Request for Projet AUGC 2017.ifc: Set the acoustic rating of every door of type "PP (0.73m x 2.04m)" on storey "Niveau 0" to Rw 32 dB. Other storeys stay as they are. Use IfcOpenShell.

First a look at what the model holds.

```python
import ifcopenshell
import ifcopenshell.util.element

model = ifcopenshell.open("Projet AUGC 2017.ifc")
print(model.schema)
storey = next(s for s in model.by_type("IfcBuildingStorey") if s.Name == "Niveau 0")
doors = [e for e in ifcopenshell.util.element.get_decomposition(storey) if e.is_a("IfcDoor")]
seen = {}
for e in doors:
    element_type = ifcopenshell.util.element.get_type(e)
    key = (element_type.Name if element_type != e and element_type else None, ifcopenshell.util.element.get_pset(e, "Pset_DoorCommon", "AcousticRating"))
    seen[key] = seen.get(key, 0) + 1
for (name, value), count in sorted(seen.items(), key=str):
    print(count, "x", name, "|", value)
```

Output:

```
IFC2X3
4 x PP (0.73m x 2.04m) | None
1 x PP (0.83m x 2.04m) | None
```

```python
import ifcopenshell
import ifcopenshell.api.pset
import ifcopenshell.util.element

model = ifcopenshell.open("Projet AUGC 2017.ifc")

storey = next(s for s in model.by_type("IfcBuildingStorey") if s.Name == "Niveau 0")
doors = [e for e in ifcopenshell.util.element.get_decomposition(storey) if e.is_a("IfcDoor")]

count = 0
for e in doors:
    element_type = ifcopenshell.util.element.get_type(e)
    if element_type in (None, e) or element_type.Name != "PP (0.73m x 2.04m)":
        continue
    # add_pset returns the element's existing set when there is one.
    pset = ifcopenshell.api.pset.add_pset(model, product=e, name="Pset_DoorCommon")
    ifcopenshell.api.pset.edit_pset(model, pset=pset, properties={"AcousticRating": "Rw 32 dB"})
    count += 1

print(count, "doors updated")

model.write("Projet AUGC 2017_updated.ifc")
```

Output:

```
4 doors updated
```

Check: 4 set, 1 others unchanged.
